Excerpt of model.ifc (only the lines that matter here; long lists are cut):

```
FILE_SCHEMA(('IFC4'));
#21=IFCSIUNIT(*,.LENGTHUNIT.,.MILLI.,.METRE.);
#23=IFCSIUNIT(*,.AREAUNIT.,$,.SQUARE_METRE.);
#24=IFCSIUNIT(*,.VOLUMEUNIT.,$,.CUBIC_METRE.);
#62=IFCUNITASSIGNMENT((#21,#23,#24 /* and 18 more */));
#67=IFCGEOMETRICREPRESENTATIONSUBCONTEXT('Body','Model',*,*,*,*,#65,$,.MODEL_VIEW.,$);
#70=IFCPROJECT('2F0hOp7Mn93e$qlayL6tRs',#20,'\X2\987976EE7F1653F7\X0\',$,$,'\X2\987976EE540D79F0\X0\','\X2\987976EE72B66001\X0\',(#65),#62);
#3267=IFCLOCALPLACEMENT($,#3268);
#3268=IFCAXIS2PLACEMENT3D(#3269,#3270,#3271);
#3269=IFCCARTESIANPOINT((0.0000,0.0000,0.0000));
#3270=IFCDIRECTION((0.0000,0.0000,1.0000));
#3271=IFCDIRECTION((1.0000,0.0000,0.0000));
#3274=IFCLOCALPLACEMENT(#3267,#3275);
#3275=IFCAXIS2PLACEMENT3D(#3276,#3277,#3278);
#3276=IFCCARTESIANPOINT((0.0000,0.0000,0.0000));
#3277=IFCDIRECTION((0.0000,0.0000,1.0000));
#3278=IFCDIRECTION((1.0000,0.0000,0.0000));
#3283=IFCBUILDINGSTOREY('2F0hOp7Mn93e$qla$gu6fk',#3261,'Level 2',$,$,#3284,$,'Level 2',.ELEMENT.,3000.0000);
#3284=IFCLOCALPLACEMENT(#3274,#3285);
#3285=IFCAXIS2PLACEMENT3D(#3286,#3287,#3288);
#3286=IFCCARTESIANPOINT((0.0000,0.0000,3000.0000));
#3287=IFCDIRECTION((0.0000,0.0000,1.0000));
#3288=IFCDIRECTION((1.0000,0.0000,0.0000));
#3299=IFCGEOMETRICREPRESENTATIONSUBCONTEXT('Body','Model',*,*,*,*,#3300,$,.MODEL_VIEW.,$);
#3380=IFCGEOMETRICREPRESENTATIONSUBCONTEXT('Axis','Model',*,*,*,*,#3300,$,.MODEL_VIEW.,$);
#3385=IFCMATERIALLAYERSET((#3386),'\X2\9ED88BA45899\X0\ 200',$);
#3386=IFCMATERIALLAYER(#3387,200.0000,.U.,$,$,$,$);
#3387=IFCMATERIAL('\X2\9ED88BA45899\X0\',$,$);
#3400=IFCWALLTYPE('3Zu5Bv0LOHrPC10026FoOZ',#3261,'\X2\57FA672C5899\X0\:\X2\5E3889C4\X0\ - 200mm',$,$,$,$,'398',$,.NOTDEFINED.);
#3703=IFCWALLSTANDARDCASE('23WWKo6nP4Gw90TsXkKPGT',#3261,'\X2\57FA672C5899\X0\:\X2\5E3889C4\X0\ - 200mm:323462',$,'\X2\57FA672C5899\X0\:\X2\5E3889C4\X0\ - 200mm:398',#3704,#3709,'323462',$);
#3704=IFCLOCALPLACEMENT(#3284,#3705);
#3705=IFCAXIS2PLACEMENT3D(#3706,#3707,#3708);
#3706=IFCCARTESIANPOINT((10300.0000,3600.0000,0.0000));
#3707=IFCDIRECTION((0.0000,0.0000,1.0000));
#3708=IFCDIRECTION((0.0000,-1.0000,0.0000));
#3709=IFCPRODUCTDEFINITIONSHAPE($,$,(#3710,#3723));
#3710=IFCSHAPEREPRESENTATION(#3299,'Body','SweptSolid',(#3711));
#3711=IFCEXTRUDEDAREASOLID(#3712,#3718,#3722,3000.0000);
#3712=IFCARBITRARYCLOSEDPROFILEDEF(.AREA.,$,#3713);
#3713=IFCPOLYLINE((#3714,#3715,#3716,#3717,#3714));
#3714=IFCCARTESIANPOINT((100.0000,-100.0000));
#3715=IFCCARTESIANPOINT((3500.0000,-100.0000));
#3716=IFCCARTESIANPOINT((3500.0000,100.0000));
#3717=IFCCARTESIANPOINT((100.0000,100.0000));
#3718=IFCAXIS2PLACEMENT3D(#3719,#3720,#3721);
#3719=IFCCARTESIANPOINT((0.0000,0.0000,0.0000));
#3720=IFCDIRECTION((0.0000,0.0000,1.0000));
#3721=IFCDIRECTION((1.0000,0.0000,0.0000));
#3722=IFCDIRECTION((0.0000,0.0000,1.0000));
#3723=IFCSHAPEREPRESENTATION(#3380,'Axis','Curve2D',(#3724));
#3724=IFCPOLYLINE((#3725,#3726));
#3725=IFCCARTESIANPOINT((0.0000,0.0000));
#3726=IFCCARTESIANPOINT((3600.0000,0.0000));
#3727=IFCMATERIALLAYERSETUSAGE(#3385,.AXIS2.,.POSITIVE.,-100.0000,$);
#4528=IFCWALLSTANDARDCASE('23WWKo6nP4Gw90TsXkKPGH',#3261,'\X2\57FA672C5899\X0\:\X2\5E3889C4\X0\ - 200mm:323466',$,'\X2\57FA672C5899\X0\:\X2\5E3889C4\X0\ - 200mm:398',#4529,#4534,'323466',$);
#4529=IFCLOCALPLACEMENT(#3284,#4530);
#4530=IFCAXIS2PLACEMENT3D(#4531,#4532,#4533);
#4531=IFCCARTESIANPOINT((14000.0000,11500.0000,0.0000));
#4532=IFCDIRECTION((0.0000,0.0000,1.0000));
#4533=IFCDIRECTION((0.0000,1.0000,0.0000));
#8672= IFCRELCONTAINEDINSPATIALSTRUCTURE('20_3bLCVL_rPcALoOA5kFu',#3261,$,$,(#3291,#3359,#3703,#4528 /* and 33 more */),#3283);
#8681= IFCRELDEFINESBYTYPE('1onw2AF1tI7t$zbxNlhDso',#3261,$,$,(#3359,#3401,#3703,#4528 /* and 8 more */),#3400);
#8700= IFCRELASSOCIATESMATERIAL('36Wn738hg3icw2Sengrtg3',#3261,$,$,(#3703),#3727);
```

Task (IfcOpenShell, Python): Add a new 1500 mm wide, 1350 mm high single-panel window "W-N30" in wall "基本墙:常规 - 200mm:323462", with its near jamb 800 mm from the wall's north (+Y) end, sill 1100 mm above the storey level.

```python
import numpy as np
import ifcopenshell
import ifcopenshell.api.feature
import ifcopenshell.api.geometry
import ifcopenshell.api.root
import ifcopenshell.api.spatial
import ifcopenshell.geom
import ifcopenshell.util.element
import ifcopenshell.util.placement
import ifcopenshell.util.representation
import ifcopenshell.util.shape
import ifcopenshell.util.unit

model = ifcopenshell.open("model.ifc")
unit_scale = ifcopenshell.util.unit.calculate_unit_scale(model)
settings = ifcopenshell.geom.settings()


def volume(element):
    """Net volume in cubic metres, openings subtracted."""
    shape = ifcopenshell.geom.create_shape(settings, element)
    return ifcopenshell.util.shape.get_volume(shape.geometry)


wall = model.by_guid("23WWKo6nP4Gw90TsXkKPGT")
storey = ifcopenshell.util.element.get_container(wall, ifc_class="IfcBuildingStorey")
context = ifcopenshell.util.representation.get_context(model, "Model", "Body", "MODEL_VIEW")
before = volume(wall)

width, height, from_end, sill = 1.5, 1.35, 0.8, 1.1  # metres

# The wall runs along its own X axis, and the end named is its -X end.
wall_shape = ifcopenshell.geom.create_shape(settings, wall)
x, y, z = ifcopenshell.util.shape.get_vertices(wall_shape.geometry).T
start = x.min() + from_end
face, thickness = float(y.min()), float(y.max() - y.min())
wall_matrix = ifcopenshell.util.placement.get_local_placement(wall.ObjectPlacement)
level = ifcopenshell.util.placement.get_local_placement(storey.ObjectPlacement)[2, 3]


def in_wall(x, y):
    """Placement at x, y metres in the wall's axes, at sill height."""
    matrix = wall_matrix.copy()
    matrix[:, 3] = wall_matrix @ np.array([x / unit_scale, y / unit_scale, 0.0, 1.0])
    matrix[2, 3] = level + sill / unit_scale
    return matrix


# Opening: a box that overshoots both wall faces by 50 mm.
opening = ifcopenshell.api.root.create_entity(model, ifc_class="IfcOpeningElement", predefined_type="OPENING")
box = ifcopenshell.api.geometry.add_wall_representation(
    model, context=context, length=width, height=height, thickness=thickness + 0.1
)
ifcopenshell.api.geometry.assign_representation(model, product=opening, representation=box)
ifcopenshell.api.geometry.edit_object_placement(model, product=opening, matrix=in_wall(start, face - 0.05), is_si=False)
ifcopenshell.api.feature.add_feature(model, feature=opening, element=wall)

window = ifcopenshell.api.root.create_entity(model, ifc_class="IfcWindow", name="W-N30", predefined_type="WINDOW")
window.OverallWidth, window.OverallHeight = width / unit_scale, height / unit_scale
window.PartitioningType = "SINGLE_PANEL"
body = ifcopenshell.api.geometry.add_window_representation(
    model,
    context=context,
    overall_width=window.OverallWidth,
    overall_height=window.OverallHeight,
    partition_type="SINGLE_PANEL",
)
ifcopenshell.api.geometry.assign_representation(model, product=window, representation=body)
ifcopenshell.api.spatial.assign_container(model, products=[window], relating_structure=storey)
ifcopenshell.api.feature.add_filling(model, opening=opening, element=window)

# Centre the window in the wall's thickness.
ifcopenshell.api.geometry.edit_object_placement(model, product=window, matrix=in_wall(start, face), is_si=False)
window_shape = ifcopenshell.geom.create_shape(settings, window)
depth = ifcopenshell.util.shape.get_vertices(window_shape.geometry)[:, 1]
offset = face + thickness / 2 - (depth.min() + depth.max()) / 2
ifcopenshell.api.geometry.edit_object_placement(model, product=window, matrix=in_wall(start, offset), is_si=False)

after = volume(wall)

print(f"wall volume {before:.3f} -> {after:.3f} m3")

model.write("model_v2.ifc")
```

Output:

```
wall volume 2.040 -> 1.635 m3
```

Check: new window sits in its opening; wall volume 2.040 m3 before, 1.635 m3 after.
